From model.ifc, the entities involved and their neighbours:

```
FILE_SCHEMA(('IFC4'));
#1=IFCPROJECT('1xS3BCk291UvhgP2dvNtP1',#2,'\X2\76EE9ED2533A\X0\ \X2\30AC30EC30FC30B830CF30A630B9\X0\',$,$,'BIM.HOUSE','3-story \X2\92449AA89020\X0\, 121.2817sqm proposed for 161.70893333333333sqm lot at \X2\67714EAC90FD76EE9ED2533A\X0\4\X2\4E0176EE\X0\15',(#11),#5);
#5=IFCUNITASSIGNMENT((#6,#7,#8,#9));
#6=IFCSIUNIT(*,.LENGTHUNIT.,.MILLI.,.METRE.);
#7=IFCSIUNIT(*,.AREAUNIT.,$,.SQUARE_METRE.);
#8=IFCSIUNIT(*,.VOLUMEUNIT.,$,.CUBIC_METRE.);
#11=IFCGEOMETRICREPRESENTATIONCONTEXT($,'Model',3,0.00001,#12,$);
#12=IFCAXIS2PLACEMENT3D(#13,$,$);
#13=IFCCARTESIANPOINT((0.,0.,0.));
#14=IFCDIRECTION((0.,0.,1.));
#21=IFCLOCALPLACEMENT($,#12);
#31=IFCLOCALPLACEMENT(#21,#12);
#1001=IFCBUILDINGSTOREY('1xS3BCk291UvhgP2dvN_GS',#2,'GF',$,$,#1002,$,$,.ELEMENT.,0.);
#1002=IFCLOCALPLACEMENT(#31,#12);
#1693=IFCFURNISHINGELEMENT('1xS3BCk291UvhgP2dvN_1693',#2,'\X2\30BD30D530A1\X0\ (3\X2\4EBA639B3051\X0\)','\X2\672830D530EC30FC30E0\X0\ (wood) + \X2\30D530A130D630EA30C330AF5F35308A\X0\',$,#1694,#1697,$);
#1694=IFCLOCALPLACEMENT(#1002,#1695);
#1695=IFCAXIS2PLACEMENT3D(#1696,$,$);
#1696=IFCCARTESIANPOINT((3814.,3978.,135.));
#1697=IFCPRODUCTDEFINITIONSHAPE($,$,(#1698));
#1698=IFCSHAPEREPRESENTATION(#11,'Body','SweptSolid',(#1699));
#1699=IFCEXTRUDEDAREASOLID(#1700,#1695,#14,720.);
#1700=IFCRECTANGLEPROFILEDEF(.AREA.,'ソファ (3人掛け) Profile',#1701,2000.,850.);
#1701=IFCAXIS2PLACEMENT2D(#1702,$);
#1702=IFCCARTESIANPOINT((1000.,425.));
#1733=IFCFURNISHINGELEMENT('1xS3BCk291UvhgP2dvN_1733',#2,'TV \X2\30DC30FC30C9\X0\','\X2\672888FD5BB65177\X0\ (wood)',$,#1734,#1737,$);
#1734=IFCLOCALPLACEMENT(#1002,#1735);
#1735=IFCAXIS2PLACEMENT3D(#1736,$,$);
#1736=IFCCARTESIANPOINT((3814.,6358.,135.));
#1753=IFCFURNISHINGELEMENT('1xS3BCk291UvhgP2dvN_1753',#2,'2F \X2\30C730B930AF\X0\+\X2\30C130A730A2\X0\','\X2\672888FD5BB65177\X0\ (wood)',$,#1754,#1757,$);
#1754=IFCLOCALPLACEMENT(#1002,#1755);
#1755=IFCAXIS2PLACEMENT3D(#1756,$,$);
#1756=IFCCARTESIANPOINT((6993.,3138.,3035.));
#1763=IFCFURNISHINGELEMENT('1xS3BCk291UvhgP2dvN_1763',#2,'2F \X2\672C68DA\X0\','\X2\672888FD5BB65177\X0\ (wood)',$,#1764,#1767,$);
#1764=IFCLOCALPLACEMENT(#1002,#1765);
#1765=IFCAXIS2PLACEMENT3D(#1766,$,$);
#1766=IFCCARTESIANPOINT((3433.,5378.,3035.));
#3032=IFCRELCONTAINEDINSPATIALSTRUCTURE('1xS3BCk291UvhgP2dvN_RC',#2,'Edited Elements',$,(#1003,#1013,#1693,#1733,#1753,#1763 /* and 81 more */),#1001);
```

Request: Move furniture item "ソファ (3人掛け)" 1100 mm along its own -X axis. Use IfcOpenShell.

```python
import ifcopenshell
import ifcopenshell.api.geometry
import ifcopenshell.util.placement
import ifcopenshell.util.unit

model = ifcopenshell.open("model.ifc")
unit_scale = ifcopenshell.util.unit.calculate_unit_scale(model)

item = model.by_guid("1xS3BCk291UvhgP2dvN_1693")
matrix = ifcopenshell.util.placement.get_local_placement(item.ObjectPlacement)
matrix[:3, 3] -= matrix[:3, 0] * 1.1 / unit_scale
ifcopenshell.api.geometry.edit_object_placement(model, product=item, matrix=matrix, is_si=False)

print(ifcopenshell.util.placement.get_local_placement(item.ObjectPlacement).round(3) + 0.0)

model.write("model-out.ifc")
```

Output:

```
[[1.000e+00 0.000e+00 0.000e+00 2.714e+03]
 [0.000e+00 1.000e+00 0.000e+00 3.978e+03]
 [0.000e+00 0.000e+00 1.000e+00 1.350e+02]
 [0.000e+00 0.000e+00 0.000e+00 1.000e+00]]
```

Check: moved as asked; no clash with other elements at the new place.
